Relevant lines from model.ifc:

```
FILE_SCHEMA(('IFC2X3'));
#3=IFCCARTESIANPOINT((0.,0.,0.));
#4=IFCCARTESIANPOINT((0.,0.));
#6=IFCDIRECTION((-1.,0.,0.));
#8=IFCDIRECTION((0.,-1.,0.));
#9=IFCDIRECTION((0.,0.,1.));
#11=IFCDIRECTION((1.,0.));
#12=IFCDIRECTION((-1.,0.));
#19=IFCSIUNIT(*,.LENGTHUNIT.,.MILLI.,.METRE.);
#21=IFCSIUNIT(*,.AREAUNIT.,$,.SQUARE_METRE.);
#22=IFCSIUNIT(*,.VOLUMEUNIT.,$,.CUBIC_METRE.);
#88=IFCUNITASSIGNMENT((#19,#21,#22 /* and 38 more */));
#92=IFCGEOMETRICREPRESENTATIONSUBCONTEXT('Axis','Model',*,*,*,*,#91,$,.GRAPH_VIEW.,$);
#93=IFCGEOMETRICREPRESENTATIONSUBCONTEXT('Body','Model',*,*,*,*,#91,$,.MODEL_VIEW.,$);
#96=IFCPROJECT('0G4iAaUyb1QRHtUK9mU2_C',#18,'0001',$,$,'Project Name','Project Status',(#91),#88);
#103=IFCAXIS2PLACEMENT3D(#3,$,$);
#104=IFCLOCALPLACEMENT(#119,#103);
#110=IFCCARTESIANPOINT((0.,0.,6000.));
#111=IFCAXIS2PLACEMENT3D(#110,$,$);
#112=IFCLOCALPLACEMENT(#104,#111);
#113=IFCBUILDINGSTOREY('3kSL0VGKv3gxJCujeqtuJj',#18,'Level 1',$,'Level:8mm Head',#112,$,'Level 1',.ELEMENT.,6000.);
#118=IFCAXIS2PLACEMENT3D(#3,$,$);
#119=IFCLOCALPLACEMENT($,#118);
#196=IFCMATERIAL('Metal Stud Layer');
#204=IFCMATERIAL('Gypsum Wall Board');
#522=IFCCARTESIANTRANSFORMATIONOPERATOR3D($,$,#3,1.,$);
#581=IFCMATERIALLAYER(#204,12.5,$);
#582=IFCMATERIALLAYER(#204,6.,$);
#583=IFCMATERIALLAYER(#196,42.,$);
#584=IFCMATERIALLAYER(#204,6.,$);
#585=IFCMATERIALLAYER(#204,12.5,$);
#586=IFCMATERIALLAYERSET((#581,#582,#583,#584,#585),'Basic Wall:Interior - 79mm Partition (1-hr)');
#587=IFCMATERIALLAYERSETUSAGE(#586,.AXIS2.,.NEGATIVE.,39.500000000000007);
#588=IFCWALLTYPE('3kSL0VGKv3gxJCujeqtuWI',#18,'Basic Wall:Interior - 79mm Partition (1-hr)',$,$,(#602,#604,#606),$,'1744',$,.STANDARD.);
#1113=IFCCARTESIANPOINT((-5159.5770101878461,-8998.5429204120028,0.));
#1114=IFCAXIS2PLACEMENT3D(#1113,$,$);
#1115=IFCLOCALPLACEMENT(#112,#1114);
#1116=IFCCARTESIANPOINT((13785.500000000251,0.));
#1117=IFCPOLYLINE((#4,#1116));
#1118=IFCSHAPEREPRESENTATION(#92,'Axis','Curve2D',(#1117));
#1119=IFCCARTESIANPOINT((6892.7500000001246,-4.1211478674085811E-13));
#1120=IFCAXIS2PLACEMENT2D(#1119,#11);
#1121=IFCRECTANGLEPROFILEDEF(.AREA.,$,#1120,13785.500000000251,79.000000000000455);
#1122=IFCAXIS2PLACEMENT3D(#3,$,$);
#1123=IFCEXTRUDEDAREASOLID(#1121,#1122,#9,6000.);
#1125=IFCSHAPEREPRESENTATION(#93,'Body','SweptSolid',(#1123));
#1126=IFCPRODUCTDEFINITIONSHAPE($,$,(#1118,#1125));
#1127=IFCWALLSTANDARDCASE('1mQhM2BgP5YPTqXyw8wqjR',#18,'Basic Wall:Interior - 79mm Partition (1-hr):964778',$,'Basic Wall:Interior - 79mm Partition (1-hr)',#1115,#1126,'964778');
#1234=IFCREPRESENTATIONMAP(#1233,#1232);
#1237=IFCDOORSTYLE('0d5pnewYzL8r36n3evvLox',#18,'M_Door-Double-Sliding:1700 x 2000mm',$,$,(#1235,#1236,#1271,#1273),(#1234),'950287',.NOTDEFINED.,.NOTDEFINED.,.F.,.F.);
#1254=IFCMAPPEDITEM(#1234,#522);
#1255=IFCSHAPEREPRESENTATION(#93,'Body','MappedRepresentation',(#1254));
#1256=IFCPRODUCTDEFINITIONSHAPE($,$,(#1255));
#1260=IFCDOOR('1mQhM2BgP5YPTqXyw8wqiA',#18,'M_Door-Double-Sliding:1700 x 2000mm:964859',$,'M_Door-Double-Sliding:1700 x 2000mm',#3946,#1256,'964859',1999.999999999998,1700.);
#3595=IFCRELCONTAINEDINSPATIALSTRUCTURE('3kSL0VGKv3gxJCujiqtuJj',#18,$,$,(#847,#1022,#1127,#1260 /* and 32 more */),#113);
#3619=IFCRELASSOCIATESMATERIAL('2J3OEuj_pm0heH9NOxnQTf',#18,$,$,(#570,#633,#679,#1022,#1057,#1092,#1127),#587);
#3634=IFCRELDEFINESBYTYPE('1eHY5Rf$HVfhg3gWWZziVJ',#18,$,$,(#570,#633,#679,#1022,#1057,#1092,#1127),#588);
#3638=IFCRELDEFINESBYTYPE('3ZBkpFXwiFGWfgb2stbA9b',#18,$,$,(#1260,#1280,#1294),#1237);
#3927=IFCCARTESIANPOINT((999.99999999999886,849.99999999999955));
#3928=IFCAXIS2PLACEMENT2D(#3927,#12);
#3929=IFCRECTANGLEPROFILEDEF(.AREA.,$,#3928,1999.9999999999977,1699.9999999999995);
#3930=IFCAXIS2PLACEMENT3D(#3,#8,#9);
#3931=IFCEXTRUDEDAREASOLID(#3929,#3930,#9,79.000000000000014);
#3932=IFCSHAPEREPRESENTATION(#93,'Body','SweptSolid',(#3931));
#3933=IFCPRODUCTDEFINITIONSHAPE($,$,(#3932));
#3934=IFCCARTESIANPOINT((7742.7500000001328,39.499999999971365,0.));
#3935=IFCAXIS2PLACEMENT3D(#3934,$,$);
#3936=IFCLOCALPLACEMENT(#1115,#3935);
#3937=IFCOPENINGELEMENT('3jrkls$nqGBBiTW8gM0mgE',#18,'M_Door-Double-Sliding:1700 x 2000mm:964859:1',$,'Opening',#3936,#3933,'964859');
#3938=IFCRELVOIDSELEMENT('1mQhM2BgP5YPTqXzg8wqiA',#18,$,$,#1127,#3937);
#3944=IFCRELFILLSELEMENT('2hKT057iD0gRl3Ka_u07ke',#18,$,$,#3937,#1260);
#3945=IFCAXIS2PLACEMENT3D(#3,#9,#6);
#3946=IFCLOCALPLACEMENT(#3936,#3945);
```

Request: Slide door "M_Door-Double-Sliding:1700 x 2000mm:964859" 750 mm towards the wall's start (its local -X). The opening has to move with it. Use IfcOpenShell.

```python
import ifcopenshell
import ifcopenshell.api.geometry
import ifcopenshell.util.placement

model = ifcopenshell.open("model.ifc")

door = model.by_guid("1mQhM2BgP5YPTqXyw8wqiA")
opening = door.FillsVoids[0].RelatingOpeningElement
wall = opening.VoidsElements[0].RelatingBuildingElement

wall_matrix = ifcopenshell.util.placement.get_local_placement(wall.ObjectPlacement)
shift = wall_matrix[:3, 0] * -750.0
before = ifcopenshell.util.placement.get_local_placement(door.ObjectPlacement)[:3, 3].copy()

# The door is placed relative to its opening, so it follows when the opening moves.
matrix = ifcopenshell.util.placement.get_local_placement(opening.ObjectPlacement)
matrix[:3, 3] += shift
ifcopenshell.api.geometry.edit_object_placement(
    model, product=opening, matrix=matrix, is_si=False, should_transform_children=True
)

after = ifcopenshell.util.placement.get_local_placement(door.ObjectPlacement)[:3, 3]
print("door moved by", (after - before).round(3) + 0.0)

model.write("model_v2.ifc")
```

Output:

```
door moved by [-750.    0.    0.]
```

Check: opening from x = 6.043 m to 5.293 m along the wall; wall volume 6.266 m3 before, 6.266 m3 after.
